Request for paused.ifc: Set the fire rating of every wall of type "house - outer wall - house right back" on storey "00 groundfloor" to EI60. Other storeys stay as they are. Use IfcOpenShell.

First a look at what the model holds.

```python
import ifcopenshell
import ifcopenshell.util.element

model = ifcopenshell.open("paused.ifc")
print(model.schema)
storey = next(s for s in model.by_type("IfcBuildingStorey") if s.Name == "00 groundfloor")
walls = [e for e in ifcopenshell.util.element.get_decomposition(storey) if e.is_a("IfcWall")]
seen = {}
for e in walls:
    element_type = ifcopenshell.util.element.get_type(e)
    key = (element_type.Name if element_type != e and element_type else None, ifcopenshell.util.element.get_pset(e, "Pset_WallCommon", "FireRating"))
    seen[key] = seen.get(key, 0) + 1
for (name, value), count in sorted(seen.items(), key=str):
    print(count, "x", name, "|", value)
```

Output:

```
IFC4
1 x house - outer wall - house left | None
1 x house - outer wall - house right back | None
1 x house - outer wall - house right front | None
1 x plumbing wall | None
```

```python
import ifcopenshell
import ifcopenshell.api.pset
import ifcopenshell.util.element

model = ifcopenshell.open("paused.ifc")

storey = next(s for s in model.by_type("IfcBuildingStorey") if s.Name == "00 groundfloor")
walls = [e for e in ifcopenshell.util.element.get_decomposition(storey) if e.is_a("IfcWall")]

count = 0
for e in walls:
    element_type = ifcopenshell.util.element.get_type(e)
    if element_type in (None, e) or element_type.Name != "house - outer wall - house right back":
        continue
    # add_pset returns the element's existing set when there is one.
    pset = ifcopenshell.api.pset.add_pset(model, product=e, name="Pset_WallCommon")
    ifcopenshell.api.pset.edit_pset(model, pset=pset, properties={"FireRating": "EI60"})
    count += 1

print(count, "walls updated")

model.write("paused_rev.ifc")
```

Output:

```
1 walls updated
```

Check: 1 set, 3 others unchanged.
